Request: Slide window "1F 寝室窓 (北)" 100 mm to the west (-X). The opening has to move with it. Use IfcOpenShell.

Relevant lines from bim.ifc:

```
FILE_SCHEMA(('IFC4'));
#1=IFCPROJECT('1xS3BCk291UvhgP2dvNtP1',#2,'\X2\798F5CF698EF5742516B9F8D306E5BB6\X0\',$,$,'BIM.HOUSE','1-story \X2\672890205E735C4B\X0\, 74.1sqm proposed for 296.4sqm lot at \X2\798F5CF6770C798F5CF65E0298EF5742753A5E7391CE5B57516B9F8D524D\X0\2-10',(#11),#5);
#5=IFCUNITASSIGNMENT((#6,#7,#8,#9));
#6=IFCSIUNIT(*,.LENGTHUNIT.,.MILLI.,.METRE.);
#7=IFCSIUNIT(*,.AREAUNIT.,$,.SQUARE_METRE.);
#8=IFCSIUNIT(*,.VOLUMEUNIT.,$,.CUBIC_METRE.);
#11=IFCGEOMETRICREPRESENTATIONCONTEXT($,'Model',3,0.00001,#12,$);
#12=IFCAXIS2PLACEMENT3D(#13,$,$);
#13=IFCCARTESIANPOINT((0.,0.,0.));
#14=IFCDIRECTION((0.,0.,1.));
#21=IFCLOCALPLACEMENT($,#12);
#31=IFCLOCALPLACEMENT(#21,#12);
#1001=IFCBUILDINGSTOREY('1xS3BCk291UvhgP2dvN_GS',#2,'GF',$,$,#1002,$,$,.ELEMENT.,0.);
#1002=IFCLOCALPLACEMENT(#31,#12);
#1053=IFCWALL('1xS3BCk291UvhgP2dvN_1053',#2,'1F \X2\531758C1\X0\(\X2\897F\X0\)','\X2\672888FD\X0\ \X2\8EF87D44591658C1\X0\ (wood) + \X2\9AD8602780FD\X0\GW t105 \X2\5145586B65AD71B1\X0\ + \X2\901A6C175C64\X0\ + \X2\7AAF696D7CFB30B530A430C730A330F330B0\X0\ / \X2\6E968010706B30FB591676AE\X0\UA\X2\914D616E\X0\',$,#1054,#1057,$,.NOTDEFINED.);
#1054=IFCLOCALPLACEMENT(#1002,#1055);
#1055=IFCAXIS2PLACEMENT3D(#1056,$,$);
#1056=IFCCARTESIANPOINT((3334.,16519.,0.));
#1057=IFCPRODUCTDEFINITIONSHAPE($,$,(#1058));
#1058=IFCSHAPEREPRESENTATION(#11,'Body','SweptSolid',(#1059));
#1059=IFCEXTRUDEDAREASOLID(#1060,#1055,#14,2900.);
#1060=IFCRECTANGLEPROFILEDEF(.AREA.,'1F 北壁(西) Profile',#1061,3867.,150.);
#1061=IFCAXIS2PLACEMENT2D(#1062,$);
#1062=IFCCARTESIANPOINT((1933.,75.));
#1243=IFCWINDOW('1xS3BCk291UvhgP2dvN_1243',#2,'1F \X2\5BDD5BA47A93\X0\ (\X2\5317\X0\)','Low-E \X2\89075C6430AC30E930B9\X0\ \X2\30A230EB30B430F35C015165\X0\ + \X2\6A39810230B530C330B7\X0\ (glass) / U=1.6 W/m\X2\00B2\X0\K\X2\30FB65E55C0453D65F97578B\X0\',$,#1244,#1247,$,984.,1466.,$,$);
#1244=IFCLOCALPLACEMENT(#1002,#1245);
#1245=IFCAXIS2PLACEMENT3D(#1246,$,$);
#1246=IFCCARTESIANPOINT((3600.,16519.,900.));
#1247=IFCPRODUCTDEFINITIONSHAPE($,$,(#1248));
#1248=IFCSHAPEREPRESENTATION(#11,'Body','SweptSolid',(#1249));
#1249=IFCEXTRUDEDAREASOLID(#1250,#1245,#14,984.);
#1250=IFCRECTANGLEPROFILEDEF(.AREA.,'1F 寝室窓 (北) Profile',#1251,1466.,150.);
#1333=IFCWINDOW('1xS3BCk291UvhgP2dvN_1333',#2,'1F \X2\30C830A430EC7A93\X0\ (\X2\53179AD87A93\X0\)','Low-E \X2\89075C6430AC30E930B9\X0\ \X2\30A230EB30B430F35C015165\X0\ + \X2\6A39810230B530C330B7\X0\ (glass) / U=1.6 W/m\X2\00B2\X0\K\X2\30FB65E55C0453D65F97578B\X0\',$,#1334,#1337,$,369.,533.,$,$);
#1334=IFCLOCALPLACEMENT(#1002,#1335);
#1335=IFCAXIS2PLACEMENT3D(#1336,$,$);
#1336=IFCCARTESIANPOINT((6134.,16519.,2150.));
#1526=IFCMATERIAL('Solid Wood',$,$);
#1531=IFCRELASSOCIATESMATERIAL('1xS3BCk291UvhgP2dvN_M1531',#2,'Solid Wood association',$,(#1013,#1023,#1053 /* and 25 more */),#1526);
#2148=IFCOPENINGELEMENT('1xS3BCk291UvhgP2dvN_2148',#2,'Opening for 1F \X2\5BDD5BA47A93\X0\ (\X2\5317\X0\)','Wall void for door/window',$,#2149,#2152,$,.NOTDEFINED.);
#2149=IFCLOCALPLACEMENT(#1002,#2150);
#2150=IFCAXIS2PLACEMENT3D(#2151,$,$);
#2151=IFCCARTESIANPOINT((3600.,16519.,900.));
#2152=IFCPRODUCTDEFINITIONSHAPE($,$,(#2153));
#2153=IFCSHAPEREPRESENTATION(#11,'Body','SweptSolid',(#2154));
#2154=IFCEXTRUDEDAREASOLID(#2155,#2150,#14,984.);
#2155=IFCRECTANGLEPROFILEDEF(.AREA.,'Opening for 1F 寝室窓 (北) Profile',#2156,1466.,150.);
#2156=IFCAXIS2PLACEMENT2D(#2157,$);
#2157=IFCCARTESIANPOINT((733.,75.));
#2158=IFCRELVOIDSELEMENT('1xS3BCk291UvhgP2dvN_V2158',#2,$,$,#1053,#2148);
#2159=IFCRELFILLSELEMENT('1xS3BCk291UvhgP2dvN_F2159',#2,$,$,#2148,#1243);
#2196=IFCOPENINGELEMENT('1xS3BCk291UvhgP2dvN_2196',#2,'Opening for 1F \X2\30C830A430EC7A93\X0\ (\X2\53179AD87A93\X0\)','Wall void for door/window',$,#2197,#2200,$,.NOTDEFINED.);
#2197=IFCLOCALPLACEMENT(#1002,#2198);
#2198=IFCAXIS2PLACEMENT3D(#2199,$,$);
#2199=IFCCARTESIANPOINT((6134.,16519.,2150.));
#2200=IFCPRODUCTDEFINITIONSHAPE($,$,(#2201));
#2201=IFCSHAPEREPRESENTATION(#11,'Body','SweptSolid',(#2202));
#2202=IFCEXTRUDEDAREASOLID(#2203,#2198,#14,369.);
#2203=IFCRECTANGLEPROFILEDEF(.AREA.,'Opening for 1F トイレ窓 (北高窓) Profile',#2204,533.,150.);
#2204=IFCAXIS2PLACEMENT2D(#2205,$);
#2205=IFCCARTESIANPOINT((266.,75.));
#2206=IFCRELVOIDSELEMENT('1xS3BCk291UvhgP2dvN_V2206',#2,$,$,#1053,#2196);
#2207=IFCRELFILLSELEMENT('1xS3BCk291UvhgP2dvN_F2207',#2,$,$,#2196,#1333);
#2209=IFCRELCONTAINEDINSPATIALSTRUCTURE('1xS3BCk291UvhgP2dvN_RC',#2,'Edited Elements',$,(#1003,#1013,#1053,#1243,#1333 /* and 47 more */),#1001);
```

```python
import ifcopenshell
import ifcopenshell.api.geometry
import ifcopenshell.util.placement
import ifcopenshell.util.unit

model = ifcopenshell.open("bim.ifc")
unit_scale = ifcopenshell.util.unit.calculate_unit_scale(model)

window = model.by_guid("1xS3BCk291UvhgP2dvN_1243")
opening = window.FillsVoids[0].RelatingOpeningElement
wall = opening.VoidsElements[0].RelatingBuildingElement

wall_matrix = ifcopenshell.util.placement.get_local_placement(wall.ObjectPlacement)
shift = wall_matrix[:3, 0] * -0.1 / unit_scale
before = ifcopenshell.util.placement.get_local_placement(window.ObjectPlacement)[:3, 3].copy()

# The window is not placed relative to its opening, so move both.
for product in (opening, window):
    matrix = ifcopenshell.util.placement.get_local_placement(product.ObjectPlacement)
    matrix[:3, 3] += shift
    ifcopenshell.api.geometry.edit_object_placement(model, product=product, matrix=matrix, is_si=False)

after = ifcopenshell.util.placement.get_local_placement(window.ObjectPlacement)[:3, 3]
print("window moved by", (after - before).round(3) + 0.0)

model.write("bim-out.ifc")
```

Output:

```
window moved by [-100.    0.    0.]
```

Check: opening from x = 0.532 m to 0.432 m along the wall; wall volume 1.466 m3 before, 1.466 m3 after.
